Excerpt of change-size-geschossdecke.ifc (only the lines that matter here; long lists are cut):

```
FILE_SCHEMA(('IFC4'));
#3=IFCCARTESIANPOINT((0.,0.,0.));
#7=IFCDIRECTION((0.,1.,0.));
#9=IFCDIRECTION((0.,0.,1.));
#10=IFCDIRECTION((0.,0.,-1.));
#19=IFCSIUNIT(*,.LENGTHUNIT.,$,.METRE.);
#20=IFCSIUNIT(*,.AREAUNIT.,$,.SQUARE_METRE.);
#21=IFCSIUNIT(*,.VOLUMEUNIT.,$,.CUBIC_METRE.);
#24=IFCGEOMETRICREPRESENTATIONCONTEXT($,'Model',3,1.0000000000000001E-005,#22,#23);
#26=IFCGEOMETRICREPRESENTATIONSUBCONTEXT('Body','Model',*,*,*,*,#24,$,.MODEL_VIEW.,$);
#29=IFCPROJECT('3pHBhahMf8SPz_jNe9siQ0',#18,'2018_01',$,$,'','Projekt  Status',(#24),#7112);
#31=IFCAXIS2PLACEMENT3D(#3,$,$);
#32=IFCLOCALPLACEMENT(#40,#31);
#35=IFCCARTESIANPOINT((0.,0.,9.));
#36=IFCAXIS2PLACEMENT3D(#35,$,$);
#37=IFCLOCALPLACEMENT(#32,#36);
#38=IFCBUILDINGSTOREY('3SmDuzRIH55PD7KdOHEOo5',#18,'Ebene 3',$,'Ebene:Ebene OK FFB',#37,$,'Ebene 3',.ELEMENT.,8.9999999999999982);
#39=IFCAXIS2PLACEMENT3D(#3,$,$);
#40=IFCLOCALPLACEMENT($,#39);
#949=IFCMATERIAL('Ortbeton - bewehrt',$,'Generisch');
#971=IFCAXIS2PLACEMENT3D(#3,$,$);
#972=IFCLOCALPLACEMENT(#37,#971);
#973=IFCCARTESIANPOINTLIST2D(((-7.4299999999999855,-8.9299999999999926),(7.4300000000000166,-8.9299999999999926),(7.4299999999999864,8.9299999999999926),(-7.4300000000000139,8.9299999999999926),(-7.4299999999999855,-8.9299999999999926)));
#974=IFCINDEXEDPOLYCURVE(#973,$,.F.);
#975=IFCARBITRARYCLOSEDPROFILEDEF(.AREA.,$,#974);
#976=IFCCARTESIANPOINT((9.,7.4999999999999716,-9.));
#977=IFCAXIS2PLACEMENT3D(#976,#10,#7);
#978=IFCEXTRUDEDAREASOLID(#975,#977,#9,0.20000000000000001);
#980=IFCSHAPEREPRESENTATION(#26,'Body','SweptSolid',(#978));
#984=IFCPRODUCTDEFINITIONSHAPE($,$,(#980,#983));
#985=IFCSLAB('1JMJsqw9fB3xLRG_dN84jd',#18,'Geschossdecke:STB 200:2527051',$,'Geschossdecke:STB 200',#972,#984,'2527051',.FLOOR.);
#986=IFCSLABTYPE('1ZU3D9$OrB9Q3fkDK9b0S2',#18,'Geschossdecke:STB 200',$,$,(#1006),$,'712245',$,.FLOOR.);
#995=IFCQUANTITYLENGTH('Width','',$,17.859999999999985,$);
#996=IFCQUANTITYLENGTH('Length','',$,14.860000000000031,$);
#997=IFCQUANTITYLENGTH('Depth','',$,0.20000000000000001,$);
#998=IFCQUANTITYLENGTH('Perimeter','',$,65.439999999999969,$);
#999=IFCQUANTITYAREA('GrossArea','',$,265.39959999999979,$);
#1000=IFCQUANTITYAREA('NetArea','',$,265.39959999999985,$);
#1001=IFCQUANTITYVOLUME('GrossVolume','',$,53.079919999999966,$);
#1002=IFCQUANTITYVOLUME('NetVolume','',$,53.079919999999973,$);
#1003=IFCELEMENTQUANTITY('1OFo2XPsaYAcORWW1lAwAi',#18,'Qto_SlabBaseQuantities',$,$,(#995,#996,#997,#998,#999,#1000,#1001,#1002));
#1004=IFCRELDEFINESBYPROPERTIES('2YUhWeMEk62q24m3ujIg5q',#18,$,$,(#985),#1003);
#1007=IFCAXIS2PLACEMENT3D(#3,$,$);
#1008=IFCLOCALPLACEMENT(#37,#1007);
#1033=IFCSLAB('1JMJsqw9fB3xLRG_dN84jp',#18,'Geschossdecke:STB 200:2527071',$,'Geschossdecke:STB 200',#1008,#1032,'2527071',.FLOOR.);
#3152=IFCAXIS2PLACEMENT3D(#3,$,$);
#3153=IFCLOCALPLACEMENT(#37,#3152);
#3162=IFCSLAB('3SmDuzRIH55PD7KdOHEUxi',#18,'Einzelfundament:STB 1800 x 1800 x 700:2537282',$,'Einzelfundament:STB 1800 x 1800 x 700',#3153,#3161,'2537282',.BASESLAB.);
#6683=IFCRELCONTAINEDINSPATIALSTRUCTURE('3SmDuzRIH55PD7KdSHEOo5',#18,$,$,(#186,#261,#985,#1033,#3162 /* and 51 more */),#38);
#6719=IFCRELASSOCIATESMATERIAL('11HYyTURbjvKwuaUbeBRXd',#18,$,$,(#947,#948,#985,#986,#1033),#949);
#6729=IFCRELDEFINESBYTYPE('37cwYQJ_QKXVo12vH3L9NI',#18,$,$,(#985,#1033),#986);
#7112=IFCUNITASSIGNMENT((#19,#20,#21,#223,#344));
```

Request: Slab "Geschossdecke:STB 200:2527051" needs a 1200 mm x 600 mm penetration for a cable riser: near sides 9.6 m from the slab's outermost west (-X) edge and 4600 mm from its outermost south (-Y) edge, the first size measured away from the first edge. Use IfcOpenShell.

```python
import numpy as np
import ifcopenshell
import ifcopenshell.api.feature
import ifcopenshell.api.geometry
import ifcopenshell.api.pset
import ifcopenshell.api.root
import ifcopenshell.geom
import ifcopenshell.util.element
import ifcopenshell.util.placement
import ifcopenshell.util.representation
import ifcopenshell.util.shape
import ifcopenshell.util.unit

model = ifcopenshell.open("change-size-geschossdecke.ifc")
unit_scale = ifcopenshell.util.unit.calculate_unit_scale(model)
area_scale = ifcopenshell.util.unit.calculate_unit_scale(model, "AREAUNIT")
volume_scale = ifcopenshell.util.unit.calculate_unit_scale(model, "VOLUMEUNIT")
settings = ifcopenshell.geom.settings()


def volume(element):
    """Net volume in cubic metres, openings subtracted."""
    shape = ifcopenshell.geom.create_shape(settings, element)
    return ifcopenshell.util.shape.get_volume(shape.geometry)


slab = model.by_guid("1JMJsqw9fB3xLRG_dN84jd")
before = volume(slab)

# Extent in the slab's own axes, in metres. The edges named are its -X and -Y sides.
slab_shape = ifcopenshell.geom.create_shape(settings, slab)
vertices = ifcopenshell.util.shape.get_vertices(slab_shape.geometry)
x_min, y_min, bottom = vertices.min(axis=0)
top = vertices[:, 2].max()

opening = ifcopenshell.api.root.create_entity(model, ifc_class="IfcOpeningElement", name="Cable riser opening", predefined_type="OPENING")
context = ifcopenshell.util.representation.get_context(model, "Model", "Body", "MODEL_VIEW")
width, depth = 1.2, 0.6
outline = [(0.0, 0.0), (width, 0.0), (width, depth), (0.0, depth), (0.0, 0.0)]
# Overshoot both faces by 50 mm so the cut is clean.
shape = ifcopenshell.api.geometry.add_slab_representation(
    model, context=context, depth=top - bottom + 0.1, polyline=outline
)
ifcopenshell.api.geometry.assign_representation(model, product=opening, representation=shape)

matrix = ifcopenshell.util.placement.get_local_placement(slab.ObjectPlacement)
matrix[:, 3] = matrix @ np.append(np.array([x_min + 9.6, y_min + 4.6, bottom - 0.05]) / unit_scale, 1.0)
ifcopenshell.api.geometry.edit_object_placement(model, product=opening, matrix=matrix, is_si=False)
ifcopenshell.api.feature.add_feature(model, feature=opening, element=slab)

after = volume(slab)

# Update the slab's stored quantities.
qto = model.by_id(ifcopenshell.util.element.get_pset(slab, "Qto_SlabBaseQuantities", should_inherit=False)["id"])
ifcopenshell.api.pset.edit_qto(model, qto=qto, properties={
    "NetArea": after / (top - bottom) / area_scale,
    "NetVolume": after / volume_scale,
})

print(f"slab volume {before:.3f} -> {after:.3f} m3")

model.write("change-size-geschossdecke_edited.ifc")
```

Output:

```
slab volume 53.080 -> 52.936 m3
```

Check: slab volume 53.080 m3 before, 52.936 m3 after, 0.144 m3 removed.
